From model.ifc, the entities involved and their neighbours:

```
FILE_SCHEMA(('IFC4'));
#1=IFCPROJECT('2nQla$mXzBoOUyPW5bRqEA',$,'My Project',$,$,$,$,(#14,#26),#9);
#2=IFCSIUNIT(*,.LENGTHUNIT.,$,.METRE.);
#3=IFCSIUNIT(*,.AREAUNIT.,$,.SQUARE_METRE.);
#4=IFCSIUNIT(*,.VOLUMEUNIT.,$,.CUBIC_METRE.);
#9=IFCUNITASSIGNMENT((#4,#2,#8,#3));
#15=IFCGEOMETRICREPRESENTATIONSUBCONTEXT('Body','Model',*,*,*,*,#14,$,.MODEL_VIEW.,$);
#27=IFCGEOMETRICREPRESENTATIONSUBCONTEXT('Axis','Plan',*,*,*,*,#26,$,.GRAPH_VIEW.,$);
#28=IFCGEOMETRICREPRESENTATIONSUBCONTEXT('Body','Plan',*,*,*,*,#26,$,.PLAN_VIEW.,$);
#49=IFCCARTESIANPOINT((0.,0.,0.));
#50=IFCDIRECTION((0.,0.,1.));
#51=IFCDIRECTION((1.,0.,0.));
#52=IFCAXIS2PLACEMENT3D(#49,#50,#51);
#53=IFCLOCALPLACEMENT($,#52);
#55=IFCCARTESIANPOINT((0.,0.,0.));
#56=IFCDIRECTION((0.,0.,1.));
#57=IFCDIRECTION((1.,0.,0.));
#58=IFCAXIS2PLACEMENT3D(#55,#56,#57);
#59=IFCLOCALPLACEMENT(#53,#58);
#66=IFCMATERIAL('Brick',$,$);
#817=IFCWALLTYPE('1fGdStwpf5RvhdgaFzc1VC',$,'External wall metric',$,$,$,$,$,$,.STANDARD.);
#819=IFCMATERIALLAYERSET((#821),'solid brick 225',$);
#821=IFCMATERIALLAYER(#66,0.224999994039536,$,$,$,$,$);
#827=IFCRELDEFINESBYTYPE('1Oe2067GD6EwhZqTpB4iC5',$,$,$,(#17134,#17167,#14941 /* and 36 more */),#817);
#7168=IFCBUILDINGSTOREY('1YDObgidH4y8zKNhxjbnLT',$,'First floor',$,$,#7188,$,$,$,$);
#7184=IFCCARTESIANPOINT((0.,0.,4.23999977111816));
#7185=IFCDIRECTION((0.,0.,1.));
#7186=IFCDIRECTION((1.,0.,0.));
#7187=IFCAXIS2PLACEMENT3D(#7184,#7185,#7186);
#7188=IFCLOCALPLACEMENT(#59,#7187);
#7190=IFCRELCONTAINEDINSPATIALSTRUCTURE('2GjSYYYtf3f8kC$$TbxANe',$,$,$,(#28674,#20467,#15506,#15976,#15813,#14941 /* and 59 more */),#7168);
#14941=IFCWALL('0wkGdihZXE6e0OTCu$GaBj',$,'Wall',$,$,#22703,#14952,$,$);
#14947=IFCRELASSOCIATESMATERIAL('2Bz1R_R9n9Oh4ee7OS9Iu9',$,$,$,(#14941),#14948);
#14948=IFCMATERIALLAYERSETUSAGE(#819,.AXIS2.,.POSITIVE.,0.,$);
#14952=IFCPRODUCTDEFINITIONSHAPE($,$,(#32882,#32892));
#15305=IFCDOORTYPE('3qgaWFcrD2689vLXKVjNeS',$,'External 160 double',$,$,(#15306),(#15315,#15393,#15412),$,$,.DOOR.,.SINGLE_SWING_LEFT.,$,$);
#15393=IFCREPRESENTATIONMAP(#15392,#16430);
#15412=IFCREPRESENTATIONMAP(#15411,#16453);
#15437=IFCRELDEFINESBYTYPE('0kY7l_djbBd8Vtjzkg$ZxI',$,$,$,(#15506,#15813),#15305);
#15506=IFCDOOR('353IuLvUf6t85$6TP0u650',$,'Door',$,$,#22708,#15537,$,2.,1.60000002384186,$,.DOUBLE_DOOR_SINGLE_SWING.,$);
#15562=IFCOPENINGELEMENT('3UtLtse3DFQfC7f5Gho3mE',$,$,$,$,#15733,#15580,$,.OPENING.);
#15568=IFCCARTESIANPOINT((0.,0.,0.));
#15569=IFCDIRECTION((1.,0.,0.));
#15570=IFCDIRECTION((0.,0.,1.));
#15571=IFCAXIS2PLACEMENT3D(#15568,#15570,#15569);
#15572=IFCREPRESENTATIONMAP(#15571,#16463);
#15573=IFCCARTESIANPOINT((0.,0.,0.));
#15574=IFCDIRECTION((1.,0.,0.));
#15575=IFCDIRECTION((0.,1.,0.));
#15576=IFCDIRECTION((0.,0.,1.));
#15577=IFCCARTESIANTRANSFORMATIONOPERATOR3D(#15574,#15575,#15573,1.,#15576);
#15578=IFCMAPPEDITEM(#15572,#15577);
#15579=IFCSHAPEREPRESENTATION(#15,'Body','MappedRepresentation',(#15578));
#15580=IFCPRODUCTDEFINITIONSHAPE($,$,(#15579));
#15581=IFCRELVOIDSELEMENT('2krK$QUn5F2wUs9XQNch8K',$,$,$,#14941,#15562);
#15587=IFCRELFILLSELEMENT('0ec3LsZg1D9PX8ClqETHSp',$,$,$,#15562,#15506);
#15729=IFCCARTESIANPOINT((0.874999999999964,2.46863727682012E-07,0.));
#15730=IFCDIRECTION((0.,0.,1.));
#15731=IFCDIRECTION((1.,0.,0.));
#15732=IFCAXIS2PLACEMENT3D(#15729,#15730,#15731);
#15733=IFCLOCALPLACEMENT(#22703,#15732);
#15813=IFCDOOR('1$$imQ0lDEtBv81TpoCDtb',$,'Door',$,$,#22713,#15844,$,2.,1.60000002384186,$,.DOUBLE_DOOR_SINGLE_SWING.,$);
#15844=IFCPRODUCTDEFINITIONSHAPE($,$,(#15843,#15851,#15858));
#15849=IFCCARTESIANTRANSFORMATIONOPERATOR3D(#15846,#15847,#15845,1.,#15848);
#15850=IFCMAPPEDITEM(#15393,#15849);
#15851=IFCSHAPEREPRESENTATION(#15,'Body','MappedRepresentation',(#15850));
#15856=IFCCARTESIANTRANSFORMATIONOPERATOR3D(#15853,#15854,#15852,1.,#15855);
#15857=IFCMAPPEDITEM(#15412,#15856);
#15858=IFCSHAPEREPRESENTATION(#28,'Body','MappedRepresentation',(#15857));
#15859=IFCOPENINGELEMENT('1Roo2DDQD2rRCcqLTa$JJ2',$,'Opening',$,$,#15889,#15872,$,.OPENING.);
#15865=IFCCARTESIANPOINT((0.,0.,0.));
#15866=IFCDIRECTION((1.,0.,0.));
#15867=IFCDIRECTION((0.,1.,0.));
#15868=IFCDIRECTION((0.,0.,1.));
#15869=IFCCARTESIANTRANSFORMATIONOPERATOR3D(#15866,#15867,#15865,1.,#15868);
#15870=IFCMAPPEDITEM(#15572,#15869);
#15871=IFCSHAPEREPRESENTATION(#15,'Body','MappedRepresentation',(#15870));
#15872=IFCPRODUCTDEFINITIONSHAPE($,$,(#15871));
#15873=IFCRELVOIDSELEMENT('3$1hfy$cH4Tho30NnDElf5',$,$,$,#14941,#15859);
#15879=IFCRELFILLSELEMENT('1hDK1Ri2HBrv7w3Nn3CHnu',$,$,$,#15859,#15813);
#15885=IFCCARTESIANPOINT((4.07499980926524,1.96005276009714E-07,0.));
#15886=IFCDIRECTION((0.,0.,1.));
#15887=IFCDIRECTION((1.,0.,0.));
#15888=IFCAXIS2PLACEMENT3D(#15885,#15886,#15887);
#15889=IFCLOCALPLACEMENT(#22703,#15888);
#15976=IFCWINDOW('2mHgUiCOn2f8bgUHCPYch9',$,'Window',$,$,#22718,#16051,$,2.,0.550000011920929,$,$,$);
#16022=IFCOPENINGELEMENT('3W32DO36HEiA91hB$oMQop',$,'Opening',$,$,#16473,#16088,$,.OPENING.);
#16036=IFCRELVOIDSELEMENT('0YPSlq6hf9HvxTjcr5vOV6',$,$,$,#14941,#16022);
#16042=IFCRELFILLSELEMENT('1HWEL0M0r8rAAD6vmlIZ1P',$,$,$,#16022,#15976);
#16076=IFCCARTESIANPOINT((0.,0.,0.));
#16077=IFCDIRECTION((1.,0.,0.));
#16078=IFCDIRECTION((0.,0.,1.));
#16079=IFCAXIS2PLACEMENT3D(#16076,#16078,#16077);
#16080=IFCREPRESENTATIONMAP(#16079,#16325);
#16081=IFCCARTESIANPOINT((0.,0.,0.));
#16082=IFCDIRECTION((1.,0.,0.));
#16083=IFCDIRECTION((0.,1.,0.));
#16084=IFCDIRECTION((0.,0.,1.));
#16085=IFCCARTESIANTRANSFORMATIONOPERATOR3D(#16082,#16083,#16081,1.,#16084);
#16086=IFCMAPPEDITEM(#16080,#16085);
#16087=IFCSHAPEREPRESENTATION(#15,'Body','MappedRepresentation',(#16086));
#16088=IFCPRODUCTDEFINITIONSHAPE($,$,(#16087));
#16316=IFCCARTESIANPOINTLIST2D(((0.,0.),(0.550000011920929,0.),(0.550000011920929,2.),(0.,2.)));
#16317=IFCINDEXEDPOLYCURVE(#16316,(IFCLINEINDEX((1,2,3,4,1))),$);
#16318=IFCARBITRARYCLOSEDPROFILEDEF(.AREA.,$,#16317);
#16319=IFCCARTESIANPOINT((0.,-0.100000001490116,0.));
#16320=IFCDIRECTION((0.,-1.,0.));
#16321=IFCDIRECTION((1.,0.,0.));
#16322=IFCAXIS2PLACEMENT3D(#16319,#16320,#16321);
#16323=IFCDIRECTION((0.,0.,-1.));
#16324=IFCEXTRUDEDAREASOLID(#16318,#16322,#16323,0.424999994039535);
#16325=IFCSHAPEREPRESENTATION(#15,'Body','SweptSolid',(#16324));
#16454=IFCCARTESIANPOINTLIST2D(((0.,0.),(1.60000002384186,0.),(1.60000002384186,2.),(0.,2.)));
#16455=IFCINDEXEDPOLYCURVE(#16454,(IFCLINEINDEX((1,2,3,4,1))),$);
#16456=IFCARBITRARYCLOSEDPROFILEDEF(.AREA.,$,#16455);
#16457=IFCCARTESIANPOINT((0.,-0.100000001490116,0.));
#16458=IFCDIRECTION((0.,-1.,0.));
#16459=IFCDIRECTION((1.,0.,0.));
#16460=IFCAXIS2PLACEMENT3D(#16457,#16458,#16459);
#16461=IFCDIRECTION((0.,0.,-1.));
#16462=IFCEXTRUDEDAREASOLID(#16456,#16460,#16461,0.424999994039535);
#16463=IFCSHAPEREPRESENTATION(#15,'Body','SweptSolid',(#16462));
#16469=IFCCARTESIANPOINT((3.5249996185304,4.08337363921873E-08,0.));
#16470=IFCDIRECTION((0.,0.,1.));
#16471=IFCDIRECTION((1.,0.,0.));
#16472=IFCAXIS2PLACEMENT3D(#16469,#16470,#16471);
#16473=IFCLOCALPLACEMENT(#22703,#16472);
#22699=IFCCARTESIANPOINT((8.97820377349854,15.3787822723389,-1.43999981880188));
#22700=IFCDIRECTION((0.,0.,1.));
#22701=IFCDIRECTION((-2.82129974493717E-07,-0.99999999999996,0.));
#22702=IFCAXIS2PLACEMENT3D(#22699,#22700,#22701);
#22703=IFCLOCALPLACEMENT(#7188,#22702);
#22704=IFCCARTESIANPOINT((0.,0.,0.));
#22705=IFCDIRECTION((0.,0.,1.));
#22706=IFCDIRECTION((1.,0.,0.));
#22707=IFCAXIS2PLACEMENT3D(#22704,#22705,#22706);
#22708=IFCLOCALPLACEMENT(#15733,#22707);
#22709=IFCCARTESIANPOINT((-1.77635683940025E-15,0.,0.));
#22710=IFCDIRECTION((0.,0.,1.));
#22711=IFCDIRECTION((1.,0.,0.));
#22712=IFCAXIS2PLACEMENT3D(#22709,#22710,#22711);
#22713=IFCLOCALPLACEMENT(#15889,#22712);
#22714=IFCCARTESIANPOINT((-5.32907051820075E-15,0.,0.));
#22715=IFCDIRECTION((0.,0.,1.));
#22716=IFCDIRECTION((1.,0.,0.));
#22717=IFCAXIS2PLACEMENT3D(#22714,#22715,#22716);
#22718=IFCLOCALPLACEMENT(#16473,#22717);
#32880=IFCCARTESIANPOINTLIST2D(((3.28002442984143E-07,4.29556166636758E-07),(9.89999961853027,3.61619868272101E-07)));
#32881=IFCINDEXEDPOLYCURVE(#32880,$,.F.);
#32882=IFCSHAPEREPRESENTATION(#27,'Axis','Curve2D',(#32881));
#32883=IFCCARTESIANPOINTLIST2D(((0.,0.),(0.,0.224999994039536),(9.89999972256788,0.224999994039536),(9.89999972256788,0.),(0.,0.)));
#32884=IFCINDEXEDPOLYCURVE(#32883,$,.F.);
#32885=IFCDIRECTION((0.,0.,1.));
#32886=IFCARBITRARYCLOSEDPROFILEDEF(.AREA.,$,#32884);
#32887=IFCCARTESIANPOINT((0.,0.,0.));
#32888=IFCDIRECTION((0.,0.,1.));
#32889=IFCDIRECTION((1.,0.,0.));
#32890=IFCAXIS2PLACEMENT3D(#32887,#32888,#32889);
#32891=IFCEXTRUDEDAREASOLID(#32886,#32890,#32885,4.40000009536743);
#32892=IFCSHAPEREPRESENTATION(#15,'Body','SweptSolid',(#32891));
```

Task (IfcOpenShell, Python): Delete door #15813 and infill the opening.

```python
import ifcopenshell
import ifcopenshell.api.feature
import ifcopenshell.api.root
import ifcopenshell.geom
import ifcopenshell.util.shape

model = ifcopenshell.open("model.ifc")
settings = ifcopenshell.geom.settings()


def volume(element):
    """Net volume in cubic metres, openings subtracted."""
    shape = ifcopenshell.geom.create_shape(settings, element)
    return ifcopenshell.util.shape.get_volume(shape.geometry)


door = model.by_id(15813)
opening = door.FillsVoids[0].RelatingOpeningElement
wall = opening.VoidsElements[0].RelatingBuildingElement
before = volume(wall)

ifcopenshell.api.root.remove_product(model, product=door)
ifcopenshell.api.feature.remove_feature(model, feature=opening)

after = volume(wall)

print(f"wall volume {before:.3f} -> {after:.3f} m3")

model.write("model_updated.ifc")
```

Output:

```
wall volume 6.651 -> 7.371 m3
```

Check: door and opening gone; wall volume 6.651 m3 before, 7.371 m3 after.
